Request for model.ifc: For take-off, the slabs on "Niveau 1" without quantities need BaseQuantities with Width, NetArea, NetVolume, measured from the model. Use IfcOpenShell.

First a look at what the model holds.

```python
import ifcopenshell
import ifcopenshell.util.element
import ifcopenshell.util.unit

model = ifcopenshell.open("model.ifc")
print(model.schema)
for unit_type in ("LENGTHUNIT", "AREAUNIT", "VOLUMEUNIT"):
    print(unit_type, ifcopenshell.util.unit.calculate_unit_scale(model, unit_type))
storey = next(s for s in model.by_type("IfcBuildingStorey") if s.Name == "Niveau 1")
slabs = [e for e in ifcopenshell.util.element.get_decomposition(storey) if e.is_a("IfcSlab")]
for e in sorted(slabs, key=lambda e: e.id()):
    print(e.id(), e.is_a(), e.Name, list(ifcopenshell.util.element.get_psets(e, qtos_only=True)), sep=" | ")
```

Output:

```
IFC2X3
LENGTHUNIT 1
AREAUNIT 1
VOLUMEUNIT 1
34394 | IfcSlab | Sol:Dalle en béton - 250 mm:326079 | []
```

```python
import ifcopenshell
import ifcopenshell.api.pset
import ifcopenshell.geom
import ifcopenshell.util.element
import ifcopenshell.util.shape
import ifcopenshell.util.unit

model = ifcopenshell.open("model.ifc")
unit_scale = ifcopenshell.util.unit.calculate_unit_scale(model)
area_scale = ifcopenshell.util.unit.calculate_unit_scale(model, "AREAUNIT")
volume_scale = ifcopenshell.util.unit.calculate_unit_scale(model, "VOLUMEUNIT")
settings = ifcopenshell.geom.settings()

storey = next(s for s in model.by_type("IfcBuildingStorey") if s.Name == "Niveau 1")
slabs = [e for e in ifcopenshell.util.element.get_decomposition(storey) if e.is_a("IfcSlab")]

for e in sorted(slabs, key=lambda e: e.id()):
    if ifcopenshell.util.element.get_psets(e, qtos_only=True, should_inherit=False):
        continue
    # Geometry comes back in metres, in the element's own axes.
    shape = ifcopenshell.geom.create_shape(settings, e)
    values = {
        "Width": ifcopenshell.util.shape.get_z(shape.geometry) / unit_scale,
        "NetArea": ifcopenshell.util.shape.get_footprint_area(shape.geometry) / area_scale,
        "NetVolume": ifcopenshell.util.shape.get_volume(shape.geometry) / volume_scale,
    }
    qto = ifcopenshell.api.pset.add_qto(model, product=e, name="BaseQuantities")
    ifcopenshell.api.pset.edit_qto(model, qto=qto, properties=values)
    print(e.id(), {k: round(v, 3) for k, v in values.items()})

model.write("model_updated.ifc")
```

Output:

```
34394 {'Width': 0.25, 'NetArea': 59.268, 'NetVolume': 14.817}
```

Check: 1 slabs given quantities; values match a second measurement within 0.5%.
